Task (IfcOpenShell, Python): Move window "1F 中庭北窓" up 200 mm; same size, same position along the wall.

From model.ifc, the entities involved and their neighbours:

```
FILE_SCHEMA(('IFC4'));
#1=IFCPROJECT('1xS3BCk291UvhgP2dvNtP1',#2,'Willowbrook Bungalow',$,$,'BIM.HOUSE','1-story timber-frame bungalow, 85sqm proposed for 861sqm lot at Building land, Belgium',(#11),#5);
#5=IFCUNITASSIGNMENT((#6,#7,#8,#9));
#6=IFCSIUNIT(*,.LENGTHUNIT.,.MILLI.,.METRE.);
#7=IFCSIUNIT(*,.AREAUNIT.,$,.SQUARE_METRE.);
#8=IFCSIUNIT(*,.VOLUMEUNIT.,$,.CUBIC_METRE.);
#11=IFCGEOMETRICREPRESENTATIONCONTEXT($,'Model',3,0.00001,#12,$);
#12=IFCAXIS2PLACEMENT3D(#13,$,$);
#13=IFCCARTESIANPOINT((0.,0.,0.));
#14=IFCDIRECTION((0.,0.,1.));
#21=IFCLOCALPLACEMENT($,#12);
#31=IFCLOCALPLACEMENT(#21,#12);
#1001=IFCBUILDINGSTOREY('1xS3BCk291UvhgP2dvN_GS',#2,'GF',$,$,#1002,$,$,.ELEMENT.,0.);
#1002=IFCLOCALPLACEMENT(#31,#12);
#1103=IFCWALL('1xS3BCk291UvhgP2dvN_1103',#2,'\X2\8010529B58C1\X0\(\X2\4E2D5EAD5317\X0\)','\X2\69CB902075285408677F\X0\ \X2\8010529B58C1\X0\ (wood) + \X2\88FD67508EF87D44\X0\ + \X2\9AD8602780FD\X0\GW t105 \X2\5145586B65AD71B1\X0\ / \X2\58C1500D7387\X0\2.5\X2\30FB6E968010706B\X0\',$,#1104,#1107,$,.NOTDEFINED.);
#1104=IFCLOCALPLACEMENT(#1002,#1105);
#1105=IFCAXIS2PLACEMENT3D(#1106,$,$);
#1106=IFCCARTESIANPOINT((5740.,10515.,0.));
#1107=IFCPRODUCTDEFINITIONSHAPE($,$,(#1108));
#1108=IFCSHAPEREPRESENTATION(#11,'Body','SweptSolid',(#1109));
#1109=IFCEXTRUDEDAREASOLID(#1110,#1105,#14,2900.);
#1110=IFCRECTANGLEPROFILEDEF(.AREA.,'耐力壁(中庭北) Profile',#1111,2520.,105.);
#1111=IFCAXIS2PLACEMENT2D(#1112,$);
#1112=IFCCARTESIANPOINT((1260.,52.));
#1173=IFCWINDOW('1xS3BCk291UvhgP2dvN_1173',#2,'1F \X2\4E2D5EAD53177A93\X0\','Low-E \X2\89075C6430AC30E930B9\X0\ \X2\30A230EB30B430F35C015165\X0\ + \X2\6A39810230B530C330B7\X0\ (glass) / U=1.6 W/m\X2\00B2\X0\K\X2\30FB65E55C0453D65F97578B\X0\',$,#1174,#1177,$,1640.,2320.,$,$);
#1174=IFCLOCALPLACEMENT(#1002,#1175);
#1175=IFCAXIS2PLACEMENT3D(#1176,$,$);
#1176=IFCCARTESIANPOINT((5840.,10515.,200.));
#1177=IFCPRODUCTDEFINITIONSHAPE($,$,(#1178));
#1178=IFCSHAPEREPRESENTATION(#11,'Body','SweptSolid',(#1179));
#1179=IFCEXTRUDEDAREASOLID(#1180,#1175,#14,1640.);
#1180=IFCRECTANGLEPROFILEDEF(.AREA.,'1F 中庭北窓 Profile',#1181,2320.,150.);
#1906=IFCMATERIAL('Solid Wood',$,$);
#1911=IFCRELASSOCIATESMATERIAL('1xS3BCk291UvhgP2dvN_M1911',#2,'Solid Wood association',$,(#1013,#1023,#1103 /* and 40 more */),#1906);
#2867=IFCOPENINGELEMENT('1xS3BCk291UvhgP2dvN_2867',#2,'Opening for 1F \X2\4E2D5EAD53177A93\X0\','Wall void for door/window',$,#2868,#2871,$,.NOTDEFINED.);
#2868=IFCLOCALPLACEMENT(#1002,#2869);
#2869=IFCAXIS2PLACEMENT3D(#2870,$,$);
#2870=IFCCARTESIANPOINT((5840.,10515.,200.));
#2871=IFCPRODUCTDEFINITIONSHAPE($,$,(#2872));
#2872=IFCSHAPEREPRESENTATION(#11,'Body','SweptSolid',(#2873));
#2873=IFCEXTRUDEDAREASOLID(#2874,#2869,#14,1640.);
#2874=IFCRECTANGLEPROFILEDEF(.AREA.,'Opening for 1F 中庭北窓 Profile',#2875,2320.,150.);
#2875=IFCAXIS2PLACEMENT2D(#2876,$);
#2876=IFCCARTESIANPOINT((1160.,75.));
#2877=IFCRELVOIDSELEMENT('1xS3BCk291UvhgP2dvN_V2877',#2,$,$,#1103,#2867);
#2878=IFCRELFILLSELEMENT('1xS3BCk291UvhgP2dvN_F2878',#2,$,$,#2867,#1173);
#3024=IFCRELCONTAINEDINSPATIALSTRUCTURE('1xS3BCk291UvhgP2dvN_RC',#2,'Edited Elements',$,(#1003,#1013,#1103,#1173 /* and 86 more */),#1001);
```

```python
import numpy as np
import ifcopenshell
import ifcopenshell.api.geometry
import ifcopenshell.util.placement
import ifcopenshell.util.unit

model = ifcopenshell.open("model.ifc")
unit_scale = ifcopenshell.util.unit.calculate_unit_scale(model)

window = model.by_guid("1xS3BCk291UvhgP2dvN_1173")
opening = window.FillsVoids[0].RelatingOpeningElement
dz = 200.0

shift = np.array([0.0, 0.0, dz])
# The window is not placed relative to its opening, so move both.
for product in (opening, window):
    matrix = ifcopenshell.util.placement.get_local_placement(product.ObjectPlacement)
    matrix[:3, 3] += shift
    ifcopenshell.api.geometry.edit_object_placement(model, product=product, matrix=matrix, is_si=False)

print(f"moved by {dz * unit_scale:+.3f} m")

model.write("model_edited.ifc")
```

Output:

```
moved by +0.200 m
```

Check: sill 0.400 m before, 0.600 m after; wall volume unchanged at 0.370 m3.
